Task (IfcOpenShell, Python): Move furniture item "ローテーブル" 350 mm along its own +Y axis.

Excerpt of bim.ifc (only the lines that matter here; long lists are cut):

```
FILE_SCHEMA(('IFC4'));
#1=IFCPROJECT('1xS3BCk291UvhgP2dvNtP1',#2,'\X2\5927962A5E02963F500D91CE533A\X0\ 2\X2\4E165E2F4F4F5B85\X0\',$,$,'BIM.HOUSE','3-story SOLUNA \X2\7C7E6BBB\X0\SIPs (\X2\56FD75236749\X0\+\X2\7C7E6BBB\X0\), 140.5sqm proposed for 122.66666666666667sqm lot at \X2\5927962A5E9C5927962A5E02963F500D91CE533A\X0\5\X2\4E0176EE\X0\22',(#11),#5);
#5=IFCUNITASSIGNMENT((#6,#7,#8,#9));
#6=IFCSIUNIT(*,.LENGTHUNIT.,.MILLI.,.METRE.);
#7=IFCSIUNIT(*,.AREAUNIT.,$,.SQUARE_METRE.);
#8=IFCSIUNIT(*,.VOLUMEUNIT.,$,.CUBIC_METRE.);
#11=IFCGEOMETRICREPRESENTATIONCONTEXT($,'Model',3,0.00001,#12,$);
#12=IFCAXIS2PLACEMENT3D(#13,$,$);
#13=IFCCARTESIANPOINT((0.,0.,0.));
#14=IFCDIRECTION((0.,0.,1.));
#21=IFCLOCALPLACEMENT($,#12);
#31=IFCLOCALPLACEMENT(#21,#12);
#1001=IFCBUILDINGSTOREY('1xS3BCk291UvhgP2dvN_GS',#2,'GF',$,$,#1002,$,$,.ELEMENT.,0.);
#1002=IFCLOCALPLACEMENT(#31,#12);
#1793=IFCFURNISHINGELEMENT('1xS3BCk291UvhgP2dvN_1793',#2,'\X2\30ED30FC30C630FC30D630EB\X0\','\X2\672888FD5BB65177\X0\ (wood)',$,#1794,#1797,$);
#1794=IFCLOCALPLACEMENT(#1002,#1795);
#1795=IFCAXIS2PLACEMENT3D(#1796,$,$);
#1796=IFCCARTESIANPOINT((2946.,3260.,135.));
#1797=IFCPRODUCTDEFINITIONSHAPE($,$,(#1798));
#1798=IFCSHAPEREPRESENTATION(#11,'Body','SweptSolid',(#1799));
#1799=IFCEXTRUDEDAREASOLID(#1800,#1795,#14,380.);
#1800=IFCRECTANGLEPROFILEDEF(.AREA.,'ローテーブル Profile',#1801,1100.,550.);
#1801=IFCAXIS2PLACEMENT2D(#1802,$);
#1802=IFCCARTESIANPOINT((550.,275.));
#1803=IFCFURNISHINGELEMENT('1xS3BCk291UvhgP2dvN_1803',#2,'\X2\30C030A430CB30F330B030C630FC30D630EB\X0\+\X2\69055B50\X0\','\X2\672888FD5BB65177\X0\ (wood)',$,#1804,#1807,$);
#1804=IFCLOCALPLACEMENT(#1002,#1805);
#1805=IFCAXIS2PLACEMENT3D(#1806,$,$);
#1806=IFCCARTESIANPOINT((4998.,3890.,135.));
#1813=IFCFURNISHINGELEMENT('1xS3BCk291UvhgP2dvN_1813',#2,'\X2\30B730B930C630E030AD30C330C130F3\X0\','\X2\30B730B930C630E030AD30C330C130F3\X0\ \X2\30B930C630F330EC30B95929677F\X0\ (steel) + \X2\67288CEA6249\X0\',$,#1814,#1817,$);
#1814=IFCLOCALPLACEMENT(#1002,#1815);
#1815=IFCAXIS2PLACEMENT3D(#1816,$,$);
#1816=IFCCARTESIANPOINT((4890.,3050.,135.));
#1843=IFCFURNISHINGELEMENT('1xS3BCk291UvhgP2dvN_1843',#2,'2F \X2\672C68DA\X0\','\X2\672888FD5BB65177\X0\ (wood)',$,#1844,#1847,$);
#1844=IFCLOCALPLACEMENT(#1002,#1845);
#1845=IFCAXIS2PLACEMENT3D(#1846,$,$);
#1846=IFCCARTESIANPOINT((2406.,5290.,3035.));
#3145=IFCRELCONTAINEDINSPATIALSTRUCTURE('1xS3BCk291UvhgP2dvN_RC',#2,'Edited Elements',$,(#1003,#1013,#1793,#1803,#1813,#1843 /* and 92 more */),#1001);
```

```python
import ifcopenshell
import ifcopenshell.api.geometry
import ifcopenshell.util.placement

model = ifcopenshell.open("bim.ifc")

item = model.by_guid("1xS3BCk291UvhgP2dvN_1793")
matrix = ifcopenshell.util.placement.get_local_placement(item.ObjectPlacement)
matrix[:3, 3] += matrix[:3, 1] * 350.0
ifcopenshell.api.geometry.edit_object_placement(model, product=item, matrix=matrix, is_si=False)

print(ifcopenshell.util.placement.get_local_placement(item.ObjectPlacement).round(3) + 0.0)

model.write("bim_v2.ifc")
```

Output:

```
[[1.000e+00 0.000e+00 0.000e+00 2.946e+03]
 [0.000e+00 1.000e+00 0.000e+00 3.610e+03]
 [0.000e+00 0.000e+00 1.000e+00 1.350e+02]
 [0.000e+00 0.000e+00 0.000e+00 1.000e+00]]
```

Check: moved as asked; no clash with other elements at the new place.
